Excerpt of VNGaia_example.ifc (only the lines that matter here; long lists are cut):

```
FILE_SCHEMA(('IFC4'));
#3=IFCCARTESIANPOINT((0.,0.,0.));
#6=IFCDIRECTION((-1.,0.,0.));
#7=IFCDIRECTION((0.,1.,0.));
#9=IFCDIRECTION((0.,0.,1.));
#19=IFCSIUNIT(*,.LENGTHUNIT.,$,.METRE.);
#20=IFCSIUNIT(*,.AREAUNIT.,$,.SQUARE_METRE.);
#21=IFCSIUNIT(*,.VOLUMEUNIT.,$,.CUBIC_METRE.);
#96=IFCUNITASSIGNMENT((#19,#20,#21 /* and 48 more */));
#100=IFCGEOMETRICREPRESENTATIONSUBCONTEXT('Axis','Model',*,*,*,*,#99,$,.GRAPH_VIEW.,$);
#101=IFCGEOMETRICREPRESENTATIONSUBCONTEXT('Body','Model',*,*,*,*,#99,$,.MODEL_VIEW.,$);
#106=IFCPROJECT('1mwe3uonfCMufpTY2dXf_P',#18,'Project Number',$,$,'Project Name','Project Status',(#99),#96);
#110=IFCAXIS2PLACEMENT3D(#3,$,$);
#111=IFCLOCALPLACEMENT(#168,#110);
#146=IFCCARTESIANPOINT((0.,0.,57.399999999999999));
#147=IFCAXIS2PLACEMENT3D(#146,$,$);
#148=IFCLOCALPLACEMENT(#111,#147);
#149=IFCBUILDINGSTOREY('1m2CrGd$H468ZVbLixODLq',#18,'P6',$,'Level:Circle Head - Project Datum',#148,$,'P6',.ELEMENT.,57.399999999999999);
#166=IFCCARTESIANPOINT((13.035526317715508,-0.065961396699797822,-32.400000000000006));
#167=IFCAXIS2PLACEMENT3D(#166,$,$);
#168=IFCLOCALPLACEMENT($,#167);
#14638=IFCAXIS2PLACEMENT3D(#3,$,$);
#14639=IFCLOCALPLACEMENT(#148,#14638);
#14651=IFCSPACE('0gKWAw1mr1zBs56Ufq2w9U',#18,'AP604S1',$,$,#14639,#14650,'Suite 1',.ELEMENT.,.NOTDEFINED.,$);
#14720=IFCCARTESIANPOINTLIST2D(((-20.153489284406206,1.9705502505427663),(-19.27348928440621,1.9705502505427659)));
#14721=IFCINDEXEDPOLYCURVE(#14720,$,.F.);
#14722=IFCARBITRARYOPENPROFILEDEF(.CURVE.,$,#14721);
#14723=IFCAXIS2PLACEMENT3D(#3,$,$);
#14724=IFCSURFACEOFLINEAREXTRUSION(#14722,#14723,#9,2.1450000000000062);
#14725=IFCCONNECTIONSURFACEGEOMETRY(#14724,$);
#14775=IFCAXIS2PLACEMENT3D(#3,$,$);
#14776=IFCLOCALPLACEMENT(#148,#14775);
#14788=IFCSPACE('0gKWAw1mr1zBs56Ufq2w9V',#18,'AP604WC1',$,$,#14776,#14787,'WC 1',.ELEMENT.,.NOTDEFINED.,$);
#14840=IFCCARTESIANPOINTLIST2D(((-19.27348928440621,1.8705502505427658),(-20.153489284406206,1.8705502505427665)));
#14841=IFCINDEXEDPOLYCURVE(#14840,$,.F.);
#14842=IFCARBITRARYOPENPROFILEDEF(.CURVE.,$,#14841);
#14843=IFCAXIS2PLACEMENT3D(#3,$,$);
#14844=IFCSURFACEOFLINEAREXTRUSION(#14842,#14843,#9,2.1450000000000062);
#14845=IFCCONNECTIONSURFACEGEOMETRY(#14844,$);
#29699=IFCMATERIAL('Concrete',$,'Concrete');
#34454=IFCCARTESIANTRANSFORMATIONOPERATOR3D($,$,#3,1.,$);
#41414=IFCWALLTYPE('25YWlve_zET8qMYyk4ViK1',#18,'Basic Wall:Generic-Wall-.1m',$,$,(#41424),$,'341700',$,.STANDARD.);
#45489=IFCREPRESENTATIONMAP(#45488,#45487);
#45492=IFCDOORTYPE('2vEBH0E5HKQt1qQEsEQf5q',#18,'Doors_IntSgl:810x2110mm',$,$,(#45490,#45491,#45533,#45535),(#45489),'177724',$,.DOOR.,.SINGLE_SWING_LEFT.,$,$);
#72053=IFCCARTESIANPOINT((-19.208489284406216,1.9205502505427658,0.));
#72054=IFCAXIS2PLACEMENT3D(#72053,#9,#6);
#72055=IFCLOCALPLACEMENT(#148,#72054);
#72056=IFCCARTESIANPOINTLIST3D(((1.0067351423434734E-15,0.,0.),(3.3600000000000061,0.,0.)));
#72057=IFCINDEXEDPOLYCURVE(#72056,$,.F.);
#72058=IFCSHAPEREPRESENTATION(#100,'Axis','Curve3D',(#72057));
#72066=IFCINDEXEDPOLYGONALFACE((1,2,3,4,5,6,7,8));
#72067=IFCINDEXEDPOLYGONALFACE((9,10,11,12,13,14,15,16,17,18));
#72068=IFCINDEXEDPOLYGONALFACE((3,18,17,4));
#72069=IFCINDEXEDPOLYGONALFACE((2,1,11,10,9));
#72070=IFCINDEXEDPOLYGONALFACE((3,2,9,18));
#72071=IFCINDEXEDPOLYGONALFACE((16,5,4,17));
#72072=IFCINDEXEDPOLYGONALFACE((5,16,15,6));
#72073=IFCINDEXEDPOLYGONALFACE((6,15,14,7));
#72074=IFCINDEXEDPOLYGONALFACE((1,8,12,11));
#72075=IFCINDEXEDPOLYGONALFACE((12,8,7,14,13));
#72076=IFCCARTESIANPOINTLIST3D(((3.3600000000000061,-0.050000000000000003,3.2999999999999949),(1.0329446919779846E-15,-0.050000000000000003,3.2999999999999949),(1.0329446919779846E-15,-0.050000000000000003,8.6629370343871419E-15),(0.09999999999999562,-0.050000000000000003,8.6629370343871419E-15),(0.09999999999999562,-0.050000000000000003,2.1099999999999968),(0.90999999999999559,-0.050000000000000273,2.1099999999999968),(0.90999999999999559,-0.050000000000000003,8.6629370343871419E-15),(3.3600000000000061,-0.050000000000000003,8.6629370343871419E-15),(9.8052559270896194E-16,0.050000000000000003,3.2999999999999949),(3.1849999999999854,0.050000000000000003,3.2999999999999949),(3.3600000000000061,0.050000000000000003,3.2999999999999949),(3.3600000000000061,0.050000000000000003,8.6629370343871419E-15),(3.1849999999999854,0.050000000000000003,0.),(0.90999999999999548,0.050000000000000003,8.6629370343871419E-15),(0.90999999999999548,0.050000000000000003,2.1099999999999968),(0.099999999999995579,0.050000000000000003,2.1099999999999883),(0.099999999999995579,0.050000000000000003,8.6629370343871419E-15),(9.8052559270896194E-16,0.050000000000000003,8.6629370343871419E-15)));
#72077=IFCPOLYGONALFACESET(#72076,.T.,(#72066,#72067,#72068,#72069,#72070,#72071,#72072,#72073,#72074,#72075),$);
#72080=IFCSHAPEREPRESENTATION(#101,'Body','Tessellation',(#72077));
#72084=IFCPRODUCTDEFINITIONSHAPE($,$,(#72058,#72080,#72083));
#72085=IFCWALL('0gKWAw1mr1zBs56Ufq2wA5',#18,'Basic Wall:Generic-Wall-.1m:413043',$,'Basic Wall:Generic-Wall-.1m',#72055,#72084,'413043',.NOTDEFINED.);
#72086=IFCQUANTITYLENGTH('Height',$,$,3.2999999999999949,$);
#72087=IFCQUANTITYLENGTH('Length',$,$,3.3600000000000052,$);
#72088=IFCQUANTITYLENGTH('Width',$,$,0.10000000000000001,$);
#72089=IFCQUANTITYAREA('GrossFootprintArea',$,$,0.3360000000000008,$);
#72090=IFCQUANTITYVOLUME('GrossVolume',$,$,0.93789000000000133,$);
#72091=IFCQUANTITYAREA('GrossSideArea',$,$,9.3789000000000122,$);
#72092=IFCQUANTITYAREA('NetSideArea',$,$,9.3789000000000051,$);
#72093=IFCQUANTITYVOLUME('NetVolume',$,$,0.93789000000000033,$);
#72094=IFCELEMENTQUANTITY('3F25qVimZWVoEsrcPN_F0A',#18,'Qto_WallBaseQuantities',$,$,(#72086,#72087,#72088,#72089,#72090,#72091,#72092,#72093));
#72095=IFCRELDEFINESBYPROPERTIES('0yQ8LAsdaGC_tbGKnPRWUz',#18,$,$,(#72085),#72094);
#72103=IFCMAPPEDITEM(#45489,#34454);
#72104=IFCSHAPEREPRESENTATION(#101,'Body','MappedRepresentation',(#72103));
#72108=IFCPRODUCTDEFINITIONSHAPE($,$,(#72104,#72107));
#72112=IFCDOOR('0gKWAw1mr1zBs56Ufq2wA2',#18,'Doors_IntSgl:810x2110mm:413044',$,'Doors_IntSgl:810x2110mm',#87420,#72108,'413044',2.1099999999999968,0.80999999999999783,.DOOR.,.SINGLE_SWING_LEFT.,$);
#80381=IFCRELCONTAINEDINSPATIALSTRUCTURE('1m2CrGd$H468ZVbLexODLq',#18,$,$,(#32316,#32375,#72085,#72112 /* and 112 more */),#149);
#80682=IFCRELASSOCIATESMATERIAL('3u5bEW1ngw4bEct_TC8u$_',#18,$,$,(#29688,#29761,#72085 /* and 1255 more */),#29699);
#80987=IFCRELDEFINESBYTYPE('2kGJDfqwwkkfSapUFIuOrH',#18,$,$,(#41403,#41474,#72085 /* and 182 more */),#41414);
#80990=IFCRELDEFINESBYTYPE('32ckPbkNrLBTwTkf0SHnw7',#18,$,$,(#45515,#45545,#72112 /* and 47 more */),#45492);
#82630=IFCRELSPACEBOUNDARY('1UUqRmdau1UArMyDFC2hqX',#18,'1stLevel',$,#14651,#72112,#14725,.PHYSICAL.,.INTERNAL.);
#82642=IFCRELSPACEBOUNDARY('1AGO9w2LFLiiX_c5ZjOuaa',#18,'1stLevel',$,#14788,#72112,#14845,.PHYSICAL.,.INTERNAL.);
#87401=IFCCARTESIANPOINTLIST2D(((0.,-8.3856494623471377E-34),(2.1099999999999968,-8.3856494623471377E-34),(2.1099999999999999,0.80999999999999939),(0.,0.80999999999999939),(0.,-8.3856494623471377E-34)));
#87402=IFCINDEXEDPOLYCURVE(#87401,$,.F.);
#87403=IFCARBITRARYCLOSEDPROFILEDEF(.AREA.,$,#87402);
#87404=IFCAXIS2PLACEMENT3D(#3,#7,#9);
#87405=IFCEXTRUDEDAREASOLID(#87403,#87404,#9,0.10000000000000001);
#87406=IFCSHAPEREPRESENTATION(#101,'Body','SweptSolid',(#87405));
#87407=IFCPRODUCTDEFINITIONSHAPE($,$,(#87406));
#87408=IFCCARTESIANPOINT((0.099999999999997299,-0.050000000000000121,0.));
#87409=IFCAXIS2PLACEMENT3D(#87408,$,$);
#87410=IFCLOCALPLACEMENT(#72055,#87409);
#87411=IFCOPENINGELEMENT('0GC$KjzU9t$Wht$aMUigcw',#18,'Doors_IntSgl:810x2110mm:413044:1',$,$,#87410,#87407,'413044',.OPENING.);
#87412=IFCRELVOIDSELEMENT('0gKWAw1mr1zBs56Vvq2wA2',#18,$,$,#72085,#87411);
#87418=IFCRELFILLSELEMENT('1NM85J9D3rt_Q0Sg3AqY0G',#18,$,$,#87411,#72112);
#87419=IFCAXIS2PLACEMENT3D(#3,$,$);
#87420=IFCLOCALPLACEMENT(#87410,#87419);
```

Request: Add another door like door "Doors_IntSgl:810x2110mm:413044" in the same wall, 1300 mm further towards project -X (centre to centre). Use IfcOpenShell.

```python
import numpy as np
import ifcopenshell
import ifcopenshell.api.feature
import ifcopenshell.api.geometry
import ifcopenshell.api.pset
import ifcopenshell.api.root
import ifcopenshell.geom
import ifcopenshell.util.element
import ifcopenshell.util.placement
import ifcopenshell.util.shape
import ifcopenshell.util.unit

model = ifcopenshell.open("VNGaia_example.ifc")
unit_scale = ifcopenshell.util.unit.calculate_unit_scale(model)
area_scale = ifcopenshell.util.unit.calculate_unit_scale(model, "AREAUNIT")
volume_scale = ifcopenshell.util.unit.calculate_unit_scale(model, "VOLUMEUNIT")
settings = ifcopenshell.geom.settings()


def volume(element):
    """Net volume in cubic metres, openings subtracted."""
    shape = ifcopenshell.geom.create_shape(settings, element)
    return ifcopenshell.util.shape.get_volume(shape.geometry)


def reuse_history(source, copy):
    """copy_class also copies each property set's owner history, people and application; keep the originals."""
    for rel in copy.IsDefinedBy:
        if rel.is_a("IfcRelDefinesByProperties") and (history := rel.RelatingPropertyDefinition.OwnerHistory):
            rel.RelatingPropertyDefinition.OwnerHistory = source.OwnerHistory
            ifcopenshell.util.element.remove_deep2(model, history)


door = model.by_guid("0gKWAw1mr1zBs56Ufq2wA2")
opening = door.FillsVoids[0].RelatingOpeningElement
wall = opening.VoidsElements[0].RelatingBuildingElement
before = volume(wall)
shift = ifcopenshell.util.placement.get_local_placement(wall.ObjectPlacement)[:3, 0] * 1.3 / unit_scale

# copy_class copies the void relationship, type, container and properties, but no geometry.
new_opening = ifcopenshell.api.root.copy_class(model, product=opening)
new_opening.Representation = ifcopenshell.util.element.copy_deep(
    model, opening.Representation, exclude=["IfcGeometricRepresentationContext", "IfcRepresentationMap"]
)
new_opening.Name = "Doors_IntSgl:810x2110mm"
new_opening.Tag = None
reuse_history(opening, new_opening)
new_door = ifcopenshell.api.root.copy_class(model, product=door)
new_door.Representation = ifcopenshell.util.element.copy_deep(
    model, door.Representation, exclude=["IfcGeometricRepresentationContext", "IfcRepresentationMap"]
)
new_door.Name = "Doors_IntSgl:810x2110mm"
new_door.Tag = None
reuse_history(door, new_door)
ifcopenshell.api.feature.add_filling(model, opening=new_opening, element=new_door)

for old, new in ((opening, new_opening), (door, new_door)):
    matrix = ifcopenshell.util.placement.get_local_placement(old.ObjectPlacement)
    matrix[:3, 3] += shift
    ifcopenshell.api.geometry.edit_object_placement(model, product=new, matrix=matrix, is_si=False)

# The copied space boundaries still share their surfaces with the original.
for rel in new_door.ProvidesBoundaries:
    if rel.ConnectionGeometry:
        rel.ConnectionGeometry = ifcopenshell.util.element.copy_deep(model, rel.ConnectionGeometry)

# Space boundary surfaces are stored in each space's coordinates; move them too.
for rel in new_door.ProvidesBoundaries:
    if not rel.ConnectionGeometry:
        continue
    surface = rel.ConnectionGeometry.SurfaceOnRelatingElement
    space_matrix = ifcopenshell.util.placement.get_local_placement(rel.RelatingSpace.ObjectPlacement)
    point = np.array(surface.Position.Location.Coordinates) + space_matrix[:3, :3].T @ shift
    surface.Position = model.createIfcAxis2Placement3D(
        model.createIfcCartesianPoint(point.tolist()), surface.Position.Axis, surface.Position.RefDirection
    )

after = volume(wall)
thickness = 0.1  # wall thickness in metres

# Update the wall's stored quantities.
qto = model.by_id(ifcopenshell.util.element.get_pset(wall, "Qto_WallBaseQuantities", should_inherit=False)["id"])
ifcopenshell.api.pset.edit_qto(model, qto=qto, properties={
    "NetSideArea": after / thickness / area_scale,
    "NetVolume": after / volume_scale,
})

print(f"wall volume {before:.3f} -> {after:.3f} m3")

model.write("VNGaia_example-out.ifc")
```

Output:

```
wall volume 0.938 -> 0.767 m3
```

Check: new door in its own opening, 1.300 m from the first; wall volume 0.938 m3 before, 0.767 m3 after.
